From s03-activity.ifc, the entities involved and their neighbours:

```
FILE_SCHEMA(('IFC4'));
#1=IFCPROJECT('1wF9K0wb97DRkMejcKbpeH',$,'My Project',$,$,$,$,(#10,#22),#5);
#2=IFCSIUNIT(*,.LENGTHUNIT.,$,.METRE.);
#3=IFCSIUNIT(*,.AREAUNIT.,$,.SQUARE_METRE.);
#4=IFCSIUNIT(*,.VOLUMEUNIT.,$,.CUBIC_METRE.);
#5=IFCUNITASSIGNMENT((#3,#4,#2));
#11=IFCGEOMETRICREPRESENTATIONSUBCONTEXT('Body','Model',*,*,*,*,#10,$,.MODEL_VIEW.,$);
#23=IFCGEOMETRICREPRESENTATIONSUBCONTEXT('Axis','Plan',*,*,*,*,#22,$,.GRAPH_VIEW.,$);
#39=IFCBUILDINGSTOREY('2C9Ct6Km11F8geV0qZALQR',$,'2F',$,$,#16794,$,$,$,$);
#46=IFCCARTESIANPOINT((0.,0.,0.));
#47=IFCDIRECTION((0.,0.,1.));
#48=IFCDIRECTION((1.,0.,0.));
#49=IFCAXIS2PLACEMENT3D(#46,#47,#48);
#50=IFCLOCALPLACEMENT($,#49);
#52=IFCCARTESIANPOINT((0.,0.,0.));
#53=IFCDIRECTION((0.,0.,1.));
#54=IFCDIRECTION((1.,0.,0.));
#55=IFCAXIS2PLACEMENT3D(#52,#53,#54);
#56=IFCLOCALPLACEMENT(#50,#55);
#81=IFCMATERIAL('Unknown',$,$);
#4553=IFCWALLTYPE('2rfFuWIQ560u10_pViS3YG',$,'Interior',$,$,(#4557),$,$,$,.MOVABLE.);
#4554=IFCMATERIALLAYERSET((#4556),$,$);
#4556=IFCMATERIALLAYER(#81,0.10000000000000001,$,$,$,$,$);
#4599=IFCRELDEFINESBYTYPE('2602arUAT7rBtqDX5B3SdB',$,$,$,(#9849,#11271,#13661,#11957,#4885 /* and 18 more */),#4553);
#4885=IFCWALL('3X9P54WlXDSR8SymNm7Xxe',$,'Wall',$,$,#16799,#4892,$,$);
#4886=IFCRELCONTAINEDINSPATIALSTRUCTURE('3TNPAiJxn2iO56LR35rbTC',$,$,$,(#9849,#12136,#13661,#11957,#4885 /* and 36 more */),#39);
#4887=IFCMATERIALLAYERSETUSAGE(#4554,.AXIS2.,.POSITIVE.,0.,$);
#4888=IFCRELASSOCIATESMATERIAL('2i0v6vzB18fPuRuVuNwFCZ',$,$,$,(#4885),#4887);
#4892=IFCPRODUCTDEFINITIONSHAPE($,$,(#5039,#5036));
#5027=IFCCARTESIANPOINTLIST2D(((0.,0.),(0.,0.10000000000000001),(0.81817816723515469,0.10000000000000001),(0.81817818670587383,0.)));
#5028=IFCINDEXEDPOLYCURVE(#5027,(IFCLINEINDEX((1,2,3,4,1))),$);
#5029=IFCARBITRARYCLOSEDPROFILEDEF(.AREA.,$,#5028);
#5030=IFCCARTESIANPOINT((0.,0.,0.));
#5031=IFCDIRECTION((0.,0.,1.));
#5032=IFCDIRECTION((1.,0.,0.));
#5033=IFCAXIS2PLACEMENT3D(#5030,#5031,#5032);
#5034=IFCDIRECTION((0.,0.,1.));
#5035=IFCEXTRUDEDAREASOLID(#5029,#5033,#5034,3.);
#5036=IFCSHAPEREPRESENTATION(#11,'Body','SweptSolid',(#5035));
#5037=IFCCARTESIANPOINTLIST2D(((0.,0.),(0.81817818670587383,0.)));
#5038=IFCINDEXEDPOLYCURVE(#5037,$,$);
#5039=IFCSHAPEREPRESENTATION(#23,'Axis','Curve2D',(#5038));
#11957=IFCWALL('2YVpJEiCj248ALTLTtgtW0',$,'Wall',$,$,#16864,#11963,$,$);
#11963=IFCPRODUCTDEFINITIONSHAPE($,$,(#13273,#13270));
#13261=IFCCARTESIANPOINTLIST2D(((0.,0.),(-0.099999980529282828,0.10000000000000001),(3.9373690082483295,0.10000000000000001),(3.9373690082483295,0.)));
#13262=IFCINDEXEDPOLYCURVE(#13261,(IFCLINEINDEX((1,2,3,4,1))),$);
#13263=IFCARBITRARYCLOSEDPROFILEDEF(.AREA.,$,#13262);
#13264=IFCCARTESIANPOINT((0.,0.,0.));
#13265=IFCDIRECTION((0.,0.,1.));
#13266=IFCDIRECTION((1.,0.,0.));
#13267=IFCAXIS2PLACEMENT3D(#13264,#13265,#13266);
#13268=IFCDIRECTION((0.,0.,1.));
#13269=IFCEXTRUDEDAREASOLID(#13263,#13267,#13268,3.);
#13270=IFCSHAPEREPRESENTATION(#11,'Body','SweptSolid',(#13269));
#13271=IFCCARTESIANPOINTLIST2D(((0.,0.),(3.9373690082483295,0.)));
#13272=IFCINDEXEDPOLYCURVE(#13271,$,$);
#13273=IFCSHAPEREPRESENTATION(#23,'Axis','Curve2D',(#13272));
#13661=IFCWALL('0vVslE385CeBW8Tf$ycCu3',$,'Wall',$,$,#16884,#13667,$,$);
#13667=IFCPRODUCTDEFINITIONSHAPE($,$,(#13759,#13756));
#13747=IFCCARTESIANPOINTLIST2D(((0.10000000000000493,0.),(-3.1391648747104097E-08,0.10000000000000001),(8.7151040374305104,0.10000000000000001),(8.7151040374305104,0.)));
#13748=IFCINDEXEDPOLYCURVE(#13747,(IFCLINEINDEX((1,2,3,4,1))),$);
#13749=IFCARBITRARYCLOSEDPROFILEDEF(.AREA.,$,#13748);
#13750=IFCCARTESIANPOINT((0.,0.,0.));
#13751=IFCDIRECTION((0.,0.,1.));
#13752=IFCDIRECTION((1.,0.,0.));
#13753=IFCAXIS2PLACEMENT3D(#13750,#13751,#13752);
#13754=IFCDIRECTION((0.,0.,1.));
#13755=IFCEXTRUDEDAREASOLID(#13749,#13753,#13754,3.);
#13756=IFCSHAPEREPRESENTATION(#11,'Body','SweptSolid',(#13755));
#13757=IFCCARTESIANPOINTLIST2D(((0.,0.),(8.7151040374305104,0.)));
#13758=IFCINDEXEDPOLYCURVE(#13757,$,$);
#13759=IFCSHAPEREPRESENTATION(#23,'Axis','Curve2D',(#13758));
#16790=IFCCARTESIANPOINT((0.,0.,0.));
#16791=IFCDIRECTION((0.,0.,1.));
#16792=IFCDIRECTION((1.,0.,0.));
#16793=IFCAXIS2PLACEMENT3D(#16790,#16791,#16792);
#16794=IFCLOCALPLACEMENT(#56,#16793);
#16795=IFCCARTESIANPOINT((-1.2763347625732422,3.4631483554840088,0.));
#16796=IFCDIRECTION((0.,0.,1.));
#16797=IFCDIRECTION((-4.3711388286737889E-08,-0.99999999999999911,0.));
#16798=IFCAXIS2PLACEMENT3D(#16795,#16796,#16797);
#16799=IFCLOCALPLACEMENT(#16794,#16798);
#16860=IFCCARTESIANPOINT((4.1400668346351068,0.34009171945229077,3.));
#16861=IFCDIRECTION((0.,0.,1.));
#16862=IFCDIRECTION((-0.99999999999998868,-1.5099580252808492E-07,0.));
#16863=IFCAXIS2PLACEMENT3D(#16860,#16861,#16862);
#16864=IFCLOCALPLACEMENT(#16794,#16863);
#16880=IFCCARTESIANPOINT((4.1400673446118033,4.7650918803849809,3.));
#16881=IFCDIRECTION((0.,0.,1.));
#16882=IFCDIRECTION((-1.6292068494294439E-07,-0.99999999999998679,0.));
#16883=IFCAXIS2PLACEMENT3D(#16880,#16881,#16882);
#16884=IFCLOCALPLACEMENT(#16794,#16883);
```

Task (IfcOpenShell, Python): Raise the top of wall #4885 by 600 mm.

```python
import ifcopenshell
import ifcopenshell.geom
import ifcopenshell.util.representation
import ifcopenshell.util.shape
import ifcopenshell.util.unit

model = ifcopenshell.open("s03-activity.ifc")
unit_scale = ifcopenshell.util.unit.calculate_unit_scale(model)
settings = ifcopenshell.geom.settings()


def volume(element):
    """Net volume in cubic metres, openings subtracted."""
    shape = ifcopenshell.geom.create_shape(settings, element)
    return ifcopenshell.util.shape.get_volume(shape.geometry)


wall = model.by_guid("3X9P54WlXDSR8SymNm7Xxe")
before = volume(wall)

body = ifcopenshell.util.representation.get_representation(wall, "Model", "Body")
solid = body.Items[0]
old_height = solid.Depth
solid.Depth += 0.6 / unit_scale
after = volume(wall)

print(f"height {old_height:g} -> {solid.Depth:g}, volume {before:.3f} -> {after:.3f} m3")

model.write("s03-activity_edited.ifc")
```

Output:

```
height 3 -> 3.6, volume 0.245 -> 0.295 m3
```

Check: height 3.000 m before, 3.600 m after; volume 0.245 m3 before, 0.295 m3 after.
